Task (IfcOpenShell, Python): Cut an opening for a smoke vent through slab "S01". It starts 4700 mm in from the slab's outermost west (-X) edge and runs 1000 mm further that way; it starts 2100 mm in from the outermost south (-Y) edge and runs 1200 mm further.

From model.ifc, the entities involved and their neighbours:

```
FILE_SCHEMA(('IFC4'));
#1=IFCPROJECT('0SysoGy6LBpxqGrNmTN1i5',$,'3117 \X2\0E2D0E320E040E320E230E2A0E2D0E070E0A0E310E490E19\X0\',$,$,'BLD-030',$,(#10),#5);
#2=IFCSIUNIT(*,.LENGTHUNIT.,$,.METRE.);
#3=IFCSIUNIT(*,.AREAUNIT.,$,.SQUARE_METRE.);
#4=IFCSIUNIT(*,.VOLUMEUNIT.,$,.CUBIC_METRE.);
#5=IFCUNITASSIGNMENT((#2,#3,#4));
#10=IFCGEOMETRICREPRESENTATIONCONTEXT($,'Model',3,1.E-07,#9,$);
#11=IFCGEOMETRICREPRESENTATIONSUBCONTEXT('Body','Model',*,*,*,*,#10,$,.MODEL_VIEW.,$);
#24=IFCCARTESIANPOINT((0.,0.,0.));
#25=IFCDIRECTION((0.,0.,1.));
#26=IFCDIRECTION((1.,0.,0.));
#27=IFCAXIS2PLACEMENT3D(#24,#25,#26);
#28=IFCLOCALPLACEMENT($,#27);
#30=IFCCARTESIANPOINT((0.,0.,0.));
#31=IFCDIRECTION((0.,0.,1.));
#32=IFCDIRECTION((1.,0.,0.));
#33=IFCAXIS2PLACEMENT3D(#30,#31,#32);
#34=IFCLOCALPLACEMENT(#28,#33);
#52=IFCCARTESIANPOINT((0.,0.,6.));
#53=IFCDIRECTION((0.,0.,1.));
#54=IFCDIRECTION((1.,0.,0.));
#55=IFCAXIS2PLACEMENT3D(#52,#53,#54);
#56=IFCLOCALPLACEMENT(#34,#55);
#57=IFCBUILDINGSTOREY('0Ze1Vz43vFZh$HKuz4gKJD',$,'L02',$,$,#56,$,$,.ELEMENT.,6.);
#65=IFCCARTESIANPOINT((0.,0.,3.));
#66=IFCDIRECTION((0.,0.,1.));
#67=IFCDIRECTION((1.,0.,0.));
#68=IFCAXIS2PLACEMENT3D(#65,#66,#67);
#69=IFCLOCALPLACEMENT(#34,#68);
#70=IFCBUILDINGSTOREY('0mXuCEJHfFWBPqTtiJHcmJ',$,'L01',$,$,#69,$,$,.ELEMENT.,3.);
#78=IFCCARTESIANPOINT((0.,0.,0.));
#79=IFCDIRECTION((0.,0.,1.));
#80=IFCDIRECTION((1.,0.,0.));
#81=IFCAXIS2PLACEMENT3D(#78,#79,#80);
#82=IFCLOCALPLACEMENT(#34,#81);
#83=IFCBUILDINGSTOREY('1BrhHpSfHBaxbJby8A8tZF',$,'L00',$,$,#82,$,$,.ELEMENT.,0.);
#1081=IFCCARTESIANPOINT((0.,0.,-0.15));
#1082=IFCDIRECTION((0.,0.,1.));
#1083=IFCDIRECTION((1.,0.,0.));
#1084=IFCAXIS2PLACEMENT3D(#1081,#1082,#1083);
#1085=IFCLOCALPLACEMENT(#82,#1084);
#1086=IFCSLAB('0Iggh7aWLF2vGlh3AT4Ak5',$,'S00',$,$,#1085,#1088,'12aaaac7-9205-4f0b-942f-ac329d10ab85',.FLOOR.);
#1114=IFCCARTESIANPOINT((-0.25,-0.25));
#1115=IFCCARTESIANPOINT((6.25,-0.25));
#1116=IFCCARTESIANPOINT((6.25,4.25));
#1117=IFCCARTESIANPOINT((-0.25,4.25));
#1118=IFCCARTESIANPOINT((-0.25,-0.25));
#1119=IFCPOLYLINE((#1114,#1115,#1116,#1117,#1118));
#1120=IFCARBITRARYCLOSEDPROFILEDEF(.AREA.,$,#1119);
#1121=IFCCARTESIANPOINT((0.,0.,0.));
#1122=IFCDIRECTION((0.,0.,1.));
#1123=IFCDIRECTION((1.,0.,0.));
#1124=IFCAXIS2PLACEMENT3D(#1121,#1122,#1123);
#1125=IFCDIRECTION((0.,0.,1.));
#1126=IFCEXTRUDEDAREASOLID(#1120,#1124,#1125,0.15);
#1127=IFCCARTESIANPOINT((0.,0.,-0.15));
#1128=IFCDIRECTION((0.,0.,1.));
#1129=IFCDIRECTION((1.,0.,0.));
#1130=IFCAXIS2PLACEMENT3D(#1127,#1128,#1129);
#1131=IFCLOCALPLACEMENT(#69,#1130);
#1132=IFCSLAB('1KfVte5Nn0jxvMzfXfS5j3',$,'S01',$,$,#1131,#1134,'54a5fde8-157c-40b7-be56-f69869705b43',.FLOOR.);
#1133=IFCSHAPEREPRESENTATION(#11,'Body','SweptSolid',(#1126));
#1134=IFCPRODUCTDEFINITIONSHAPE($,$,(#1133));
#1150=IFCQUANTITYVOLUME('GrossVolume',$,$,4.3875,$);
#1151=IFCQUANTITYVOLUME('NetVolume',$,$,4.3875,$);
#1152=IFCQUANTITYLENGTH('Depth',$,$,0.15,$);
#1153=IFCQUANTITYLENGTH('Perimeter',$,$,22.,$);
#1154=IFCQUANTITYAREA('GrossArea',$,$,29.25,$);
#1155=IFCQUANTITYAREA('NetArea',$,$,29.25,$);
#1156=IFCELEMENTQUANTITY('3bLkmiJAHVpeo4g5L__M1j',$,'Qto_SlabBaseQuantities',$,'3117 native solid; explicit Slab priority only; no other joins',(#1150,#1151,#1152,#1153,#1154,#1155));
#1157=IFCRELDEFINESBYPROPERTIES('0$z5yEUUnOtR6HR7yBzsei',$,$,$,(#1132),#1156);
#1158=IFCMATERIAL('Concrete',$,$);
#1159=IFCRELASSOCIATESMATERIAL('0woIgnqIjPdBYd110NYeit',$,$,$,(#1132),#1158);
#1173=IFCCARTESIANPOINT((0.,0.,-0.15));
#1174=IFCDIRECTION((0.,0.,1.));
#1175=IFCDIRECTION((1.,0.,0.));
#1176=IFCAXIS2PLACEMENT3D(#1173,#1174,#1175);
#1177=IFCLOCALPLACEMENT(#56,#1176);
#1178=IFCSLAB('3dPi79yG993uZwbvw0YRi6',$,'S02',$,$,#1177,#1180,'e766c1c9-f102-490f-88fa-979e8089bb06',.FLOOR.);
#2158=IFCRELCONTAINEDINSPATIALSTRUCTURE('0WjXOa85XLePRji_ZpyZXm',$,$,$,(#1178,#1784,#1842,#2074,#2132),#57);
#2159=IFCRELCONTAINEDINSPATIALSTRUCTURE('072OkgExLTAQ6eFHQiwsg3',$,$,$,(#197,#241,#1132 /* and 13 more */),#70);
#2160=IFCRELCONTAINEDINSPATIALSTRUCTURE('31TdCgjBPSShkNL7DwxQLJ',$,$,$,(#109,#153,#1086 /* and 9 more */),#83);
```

```python
import numpy as np
import ifcopenshell
import ifcopenshell.api.feature
import ifcopenshell.api.geometry
import ifcopenshell.api.pset
import ifcopenshell.api.root
import ifcopenshell.geom
import ifcopenshell.util.element
import ifcopenshell.util.placement
import ifcopenshell.util.representation
import ifcopenshell.util.shape
import ifcopenshell.util.unit

model = ifcopenshell.open("model.ifc")
unit_scale = ifcopenshell.util.unit.calculate_unit_scale(model)
area_scale = ifcopenshell.util.unit.calculate_unit_scale(model, "AREAUNIT")
volume_scale = ifcopenshell.util.unit.calculate_unit_scale(model, "VOLUMEUNIT")
settings = ifcopenshell.geom.settings()


def volume(element):
    """Net volume in cubic metres, openings subtracted."""
    shape = ifcopenshell.geom.create_shape(settings, element)
    return ifcopenshell.util.shape.get_volume(shape.geometry)


slab = model.by_guid("1KfVte5Nn0jxvMzfXfS5j3")
before = volume(slab)

# Extent in the slab's own axes, in metres. The edges named are its -X and -Y sides.
slab_shape = ifcopenshell.geom.create_shape(settings, slab)
vertices = ifcopenshell.util.shape.get_vertices(slab_shape.geometry)
x_min, y_min, bottom = vertices.min(axis=0)
top = vertices[:, 2].max()

opening = ifcopenshell.api.root.create_entity(model, ifc_class="IfcOpeningElement", name="Smoke vent opening", predefined_type="OPENING")
context = ifcopenshell.util.representation.get_context(model, "Model", "Body", "MODEL_VIEW")
width, depth = 1, 1.2
outline = [(0.0, 0.0), (width, 0.0), (width, depth), (0.0, depth), (0.0, 0.0)]
# Overshoot both faces by 50 mm so the cut is clean.
shape = ifcopenshell.api.geometry.add_slab_representation(
    model, context=context, depth=top - bottom + 0.1, polyline=outline
)
ifcopenshell.api.geometry.assign_representation(model, product=opening, representation=shape)

matrix = ifcopenshell.util.placement.get_local_placement(slab.ObjectPlacement)
matrix[:, 3] = matrix @ np.append(np.array([x_min + 4.7, y_min + 2.1, bottom - 0.05]) / unit_scale, 1.0)
ifcopenshell.api.geometry.edit_object_placement(model, product=opening, matrix=matrix, is_si=False)
ifcopenshell.api.feature.add_feature(model, feature=opening, element=slab)

after = volume(slab)

# Update the slab's stored quantities.
qto = model.by_id(ifcopenshell.util.element.get_pset(slab, "Qto_SlabBaseQuantities", should_inherit=False)["id"])
ifcopenshell.api.pset.edit_qto(model, qto=qto, properties={
    "NetVolume": after / volume_scale,
    "NetArea": after / (top - bottom) / area_scale,
})

print(f"slab volume {before:.3f} -> {after:.3f} m3")

model.write("model_edited.ifc")
```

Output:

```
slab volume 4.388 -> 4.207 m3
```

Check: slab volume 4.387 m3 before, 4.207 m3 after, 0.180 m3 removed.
